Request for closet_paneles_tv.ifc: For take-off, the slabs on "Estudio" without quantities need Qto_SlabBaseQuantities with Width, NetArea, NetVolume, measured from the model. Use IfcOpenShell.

First a look at what the model holds.

```python
import ifcopenshell
import ifcopenshell.util.element
import ifcopenshell.util.unit

model = ifcopenshell.open("closet_paneles_tv.ifc")
print(model.schema)
for unit_type in ("LENGTHUNIT", "AREAUNIT", "VOLUMEUNIT"):
    print(unit_type, ifcopenshell.util.unit.calculate_unit_scale(model, unit_type))
storey = next(s for s in model.by_type("IfcBuildingStorey") if s.Name == "Estudio")
slabs = [e for e in ifcopenshell.util.element.get_decomposition(storey) if e.is_a("IfcSlab")]
for e in sorted(slabs, key=lambda e: e.id()):
    print(e.id(), e.is_a(), e.Name, list(ifcopenshell.util.element.get_psets(e, qtos_only=True)), sep=" | ")
```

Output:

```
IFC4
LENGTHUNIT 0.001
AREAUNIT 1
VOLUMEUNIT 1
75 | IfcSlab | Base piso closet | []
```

```python
import ifcopenshell
import ifcopenshell.api.pset
import ifcopenshell.geom
import ifcopenshell.util.element
import ifcopenshell.util.shape
import ifcopenshell.util.unit

model = ifcopenshell.open("closet_paneles_tv.ifc")
unit_scale = ifcopenshell.util.unit.calculate_unit_scale(model)
area_scale = ifcopenshell.util.unit.calculate_unit_scale(model, "AREAUNIT")
volume_scale = ifcopenshell.util.unit.calculate_unit_scale(model, "VOLUMEUNIT")
settings = ifcopenshell.geom.settings()

storey = next(s for s in model.by_type("IfcBuildingStorey") if s.Name == "Estudio")
slabs = [e for e in ifcopenshell.util.element.get_decomposition(storey) if e.is_a("IfcSlab")]

for e in sorted(slabs, key=lambda e: e.id()):
    if ifcopenshell.util.element.get_psets(e, qtos_only=True, should_inherit=False):
        continue
    # Geometry comes back in metres, in the element's own axes.
    shape = ifcopenshell.geom.create_shape(settings, e)
    values = {
        "Width": ifcopenshell.util.shape.get_z(shape.geometry) / unit_scale,
        "NetArea": ifcopenshell.util.shape.get_footprint_area(shape.geometry) / area_scale,
        "NetVolume": ifcopenshell.util.shape.get_volume(shape.geometry) / volume_scale,
    }
    qto = ifcopenshell.api.pset.add_qto(model, product=e, name="Qto_SlabBaseQuantities")
    ifcopenshell.api.pset.edit_qto(model, qto=qto, properties=values)
    print(e.id(), {k: round(v, 3) for k, v in values.items()})

model.write("closet_paneles_tv_updated.ifc")
```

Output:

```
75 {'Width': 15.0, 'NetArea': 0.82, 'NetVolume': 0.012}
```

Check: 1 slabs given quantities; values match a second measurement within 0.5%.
